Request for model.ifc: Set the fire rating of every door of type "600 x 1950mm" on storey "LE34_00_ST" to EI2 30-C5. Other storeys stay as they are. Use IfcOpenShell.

First a look at what the model holds.

```python
import ifcopenshell
import ifcopenshell.util.element

model = ifcopenshell.open("model.ifc")
print(model.schema)
storey = next(s for s in model.by_type("IfcBuildingStorey") if s.Name == "LE34_00_ST")
doors = [e for e in ifcopenshell.util.element.get_decomposition(storey) if e.is_a("IfcDoor")]
seen = {}
for e in doors:
    element_type = ifcopenshell.util.element.get_type(e)
    key = (element_type.Name if element_type != e and element_type else None, ifcopenshell.util.element.get_pset(e, "Pset_DoorCommon", "FireRating"))
    seen[key] = seen.get(key, 0) + 1
for (name, value), count in sorted(seen.items(), key=str):
    print(count, "x", name, "|", value)
```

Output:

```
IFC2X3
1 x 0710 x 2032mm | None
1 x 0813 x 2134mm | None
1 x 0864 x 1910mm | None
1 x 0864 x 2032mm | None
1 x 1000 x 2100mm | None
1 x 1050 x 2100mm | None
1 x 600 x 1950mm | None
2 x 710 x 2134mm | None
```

```python
import ifcopenshell
import ifcopenshell.api.pset
import ifcopenshell.util.element

model = ifcopenshell.open("model.ifc")

storey = next(s for s in model.by_type("IfcBuildingStorey") if s.Name == "LE34_00_ST")
doors = [e for e in ifcopenshell.util.element.get_decomposition(storey) if e.is_a("IfcDoor")]

count = 0
for e in doors:
    element_type = ifcopenshell.util.element.get_type(e)
    if element_type in (None, e) or element_type.Name != "600 x 1950mm":
        continue
    # add_pset returns the element's existing set when there is one.
    pset = ifcopenshell.api.pset.add_pset(model, product=e, name="Pset_DoorCommon")
    ifcopenshell.api.pset.edit_pset(model, pset=pset, properties={"FireRating": "EI2 30-C5"})
    count += 1

print(count, "doors updated")

model.write("model_edited.ifc")
```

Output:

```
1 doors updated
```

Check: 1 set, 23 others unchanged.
